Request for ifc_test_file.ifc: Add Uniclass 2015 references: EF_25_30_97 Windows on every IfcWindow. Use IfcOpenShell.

First a look at what the model holds.

```python
import ifcopenshell

model = ifcopenshell.open("ifc_test_file.ifc")
print(model.schema)
print("classifications:", [c.Name for c in model.by_type("IfcClassification")])
for ifc_class in ("IfcDoor", "IfcRoof", "IfcStair", "IfcWall", "IfcWindow"):
    print(ifc_class, len(model.by_type(ifc_class)))
```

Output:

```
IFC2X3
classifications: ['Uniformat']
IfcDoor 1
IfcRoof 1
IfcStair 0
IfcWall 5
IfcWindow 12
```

```python
import ifcopenshell
import ifcopenshell.api.classification

model = ifcopenshell.open("ifc_test_file.ifc")

# IFC2X3 requires Source and Edition and has no link from the project to the system.
system = model.create_entity("IfcClassification", Source="NBS", Edition="2015", Name="Uniclass 2015")

codes = {
    "IfcWindow": ("EF_25_30_97", "Windows"),
}
for ifc_class, (code, name) in codes.items():
    products = model.by_type(ifc_class)
    ifcopenshell.api.classification.add_reference(
        model, products=products, classification=system, identification=code, name=name
    )
    print(code, len(products))

model.write("ifc_test_file_v2.ifc")
```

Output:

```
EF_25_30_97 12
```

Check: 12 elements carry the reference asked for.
